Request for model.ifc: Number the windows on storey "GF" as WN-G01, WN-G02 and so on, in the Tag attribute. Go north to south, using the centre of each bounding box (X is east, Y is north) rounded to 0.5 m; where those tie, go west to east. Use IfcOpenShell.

First a look at what the model holds.

```python
import ifcopenshell
import ifcopenshell.util.element
import ifcopenshell.util.placement

model = ifcopenshell.open("model.ifc")
print(model.schema)
storey = next(s for s in model.by_type("IfcBuildingStorey") if s.Name == "GF")
windows = [e for e in ifcopenshell.util.element.get_decomposition(storey) if e.is_a("IfcWindow")]
for e in sorted(windows, key=lambda e: e.id()):
    origin = ifcopenshell.util.placement.get_local_placement(e.ObjectPlacement)[:3, 3]
    print(e.id(), e.Tag, e.Name, origin.round(2) + 0.0, sep=" | ")
```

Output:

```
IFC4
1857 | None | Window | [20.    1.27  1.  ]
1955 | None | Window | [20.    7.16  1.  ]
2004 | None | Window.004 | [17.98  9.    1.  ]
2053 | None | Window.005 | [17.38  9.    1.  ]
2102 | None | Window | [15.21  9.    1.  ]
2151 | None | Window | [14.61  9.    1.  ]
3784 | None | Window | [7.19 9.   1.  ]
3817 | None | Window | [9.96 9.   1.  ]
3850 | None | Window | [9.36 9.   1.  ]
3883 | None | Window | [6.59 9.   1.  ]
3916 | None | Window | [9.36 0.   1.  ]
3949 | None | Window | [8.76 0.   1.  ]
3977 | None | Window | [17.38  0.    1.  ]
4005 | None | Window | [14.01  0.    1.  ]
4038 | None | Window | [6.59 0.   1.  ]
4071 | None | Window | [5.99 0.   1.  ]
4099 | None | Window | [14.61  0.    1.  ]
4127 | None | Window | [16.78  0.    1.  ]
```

```python
import ifcopenshell
import ifcopenshell.geom
import ifcopenshell.util.element
import ifcopenshell.util.shape

model = ifcopenshell.open("model.ifc")
settings = ifcopenshell.geom.settings()
settings.set("use-world-coords", True)


def centre(element):
    shape = ifcopenshell.geom.create_shape(settings, element)
    return ifcopenshell.util.shape.get_bbox_centroid(shape.geometry)


storey = next(s for s in model.by_type("IfcBuildingStorey") if s.Name == "GF")
windows = [e for e in ifcopenshell.util.element.get_decomposition(storey) if e.is_a("IfcWindow")]

# Insertion points can sit at a corner or the storey origin, so sort by the geometry (in metres).
centres = {e: centre(e) for e in windows}
windows.sort(key=lambda e: (-round(centres[e][1] / 0.5), centres[e][0]))

for i, e in enumerate(windows, start=1):
    number = f"WN-G{i:02d}"
    e.Tag = number
    print(e.id(), number)

model.write("model-out.ifc")
```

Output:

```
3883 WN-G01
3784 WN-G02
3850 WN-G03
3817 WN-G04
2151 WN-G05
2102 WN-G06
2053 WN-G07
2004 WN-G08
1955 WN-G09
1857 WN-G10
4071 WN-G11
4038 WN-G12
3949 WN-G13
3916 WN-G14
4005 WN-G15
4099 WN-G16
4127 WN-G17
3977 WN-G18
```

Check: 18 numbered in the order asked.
